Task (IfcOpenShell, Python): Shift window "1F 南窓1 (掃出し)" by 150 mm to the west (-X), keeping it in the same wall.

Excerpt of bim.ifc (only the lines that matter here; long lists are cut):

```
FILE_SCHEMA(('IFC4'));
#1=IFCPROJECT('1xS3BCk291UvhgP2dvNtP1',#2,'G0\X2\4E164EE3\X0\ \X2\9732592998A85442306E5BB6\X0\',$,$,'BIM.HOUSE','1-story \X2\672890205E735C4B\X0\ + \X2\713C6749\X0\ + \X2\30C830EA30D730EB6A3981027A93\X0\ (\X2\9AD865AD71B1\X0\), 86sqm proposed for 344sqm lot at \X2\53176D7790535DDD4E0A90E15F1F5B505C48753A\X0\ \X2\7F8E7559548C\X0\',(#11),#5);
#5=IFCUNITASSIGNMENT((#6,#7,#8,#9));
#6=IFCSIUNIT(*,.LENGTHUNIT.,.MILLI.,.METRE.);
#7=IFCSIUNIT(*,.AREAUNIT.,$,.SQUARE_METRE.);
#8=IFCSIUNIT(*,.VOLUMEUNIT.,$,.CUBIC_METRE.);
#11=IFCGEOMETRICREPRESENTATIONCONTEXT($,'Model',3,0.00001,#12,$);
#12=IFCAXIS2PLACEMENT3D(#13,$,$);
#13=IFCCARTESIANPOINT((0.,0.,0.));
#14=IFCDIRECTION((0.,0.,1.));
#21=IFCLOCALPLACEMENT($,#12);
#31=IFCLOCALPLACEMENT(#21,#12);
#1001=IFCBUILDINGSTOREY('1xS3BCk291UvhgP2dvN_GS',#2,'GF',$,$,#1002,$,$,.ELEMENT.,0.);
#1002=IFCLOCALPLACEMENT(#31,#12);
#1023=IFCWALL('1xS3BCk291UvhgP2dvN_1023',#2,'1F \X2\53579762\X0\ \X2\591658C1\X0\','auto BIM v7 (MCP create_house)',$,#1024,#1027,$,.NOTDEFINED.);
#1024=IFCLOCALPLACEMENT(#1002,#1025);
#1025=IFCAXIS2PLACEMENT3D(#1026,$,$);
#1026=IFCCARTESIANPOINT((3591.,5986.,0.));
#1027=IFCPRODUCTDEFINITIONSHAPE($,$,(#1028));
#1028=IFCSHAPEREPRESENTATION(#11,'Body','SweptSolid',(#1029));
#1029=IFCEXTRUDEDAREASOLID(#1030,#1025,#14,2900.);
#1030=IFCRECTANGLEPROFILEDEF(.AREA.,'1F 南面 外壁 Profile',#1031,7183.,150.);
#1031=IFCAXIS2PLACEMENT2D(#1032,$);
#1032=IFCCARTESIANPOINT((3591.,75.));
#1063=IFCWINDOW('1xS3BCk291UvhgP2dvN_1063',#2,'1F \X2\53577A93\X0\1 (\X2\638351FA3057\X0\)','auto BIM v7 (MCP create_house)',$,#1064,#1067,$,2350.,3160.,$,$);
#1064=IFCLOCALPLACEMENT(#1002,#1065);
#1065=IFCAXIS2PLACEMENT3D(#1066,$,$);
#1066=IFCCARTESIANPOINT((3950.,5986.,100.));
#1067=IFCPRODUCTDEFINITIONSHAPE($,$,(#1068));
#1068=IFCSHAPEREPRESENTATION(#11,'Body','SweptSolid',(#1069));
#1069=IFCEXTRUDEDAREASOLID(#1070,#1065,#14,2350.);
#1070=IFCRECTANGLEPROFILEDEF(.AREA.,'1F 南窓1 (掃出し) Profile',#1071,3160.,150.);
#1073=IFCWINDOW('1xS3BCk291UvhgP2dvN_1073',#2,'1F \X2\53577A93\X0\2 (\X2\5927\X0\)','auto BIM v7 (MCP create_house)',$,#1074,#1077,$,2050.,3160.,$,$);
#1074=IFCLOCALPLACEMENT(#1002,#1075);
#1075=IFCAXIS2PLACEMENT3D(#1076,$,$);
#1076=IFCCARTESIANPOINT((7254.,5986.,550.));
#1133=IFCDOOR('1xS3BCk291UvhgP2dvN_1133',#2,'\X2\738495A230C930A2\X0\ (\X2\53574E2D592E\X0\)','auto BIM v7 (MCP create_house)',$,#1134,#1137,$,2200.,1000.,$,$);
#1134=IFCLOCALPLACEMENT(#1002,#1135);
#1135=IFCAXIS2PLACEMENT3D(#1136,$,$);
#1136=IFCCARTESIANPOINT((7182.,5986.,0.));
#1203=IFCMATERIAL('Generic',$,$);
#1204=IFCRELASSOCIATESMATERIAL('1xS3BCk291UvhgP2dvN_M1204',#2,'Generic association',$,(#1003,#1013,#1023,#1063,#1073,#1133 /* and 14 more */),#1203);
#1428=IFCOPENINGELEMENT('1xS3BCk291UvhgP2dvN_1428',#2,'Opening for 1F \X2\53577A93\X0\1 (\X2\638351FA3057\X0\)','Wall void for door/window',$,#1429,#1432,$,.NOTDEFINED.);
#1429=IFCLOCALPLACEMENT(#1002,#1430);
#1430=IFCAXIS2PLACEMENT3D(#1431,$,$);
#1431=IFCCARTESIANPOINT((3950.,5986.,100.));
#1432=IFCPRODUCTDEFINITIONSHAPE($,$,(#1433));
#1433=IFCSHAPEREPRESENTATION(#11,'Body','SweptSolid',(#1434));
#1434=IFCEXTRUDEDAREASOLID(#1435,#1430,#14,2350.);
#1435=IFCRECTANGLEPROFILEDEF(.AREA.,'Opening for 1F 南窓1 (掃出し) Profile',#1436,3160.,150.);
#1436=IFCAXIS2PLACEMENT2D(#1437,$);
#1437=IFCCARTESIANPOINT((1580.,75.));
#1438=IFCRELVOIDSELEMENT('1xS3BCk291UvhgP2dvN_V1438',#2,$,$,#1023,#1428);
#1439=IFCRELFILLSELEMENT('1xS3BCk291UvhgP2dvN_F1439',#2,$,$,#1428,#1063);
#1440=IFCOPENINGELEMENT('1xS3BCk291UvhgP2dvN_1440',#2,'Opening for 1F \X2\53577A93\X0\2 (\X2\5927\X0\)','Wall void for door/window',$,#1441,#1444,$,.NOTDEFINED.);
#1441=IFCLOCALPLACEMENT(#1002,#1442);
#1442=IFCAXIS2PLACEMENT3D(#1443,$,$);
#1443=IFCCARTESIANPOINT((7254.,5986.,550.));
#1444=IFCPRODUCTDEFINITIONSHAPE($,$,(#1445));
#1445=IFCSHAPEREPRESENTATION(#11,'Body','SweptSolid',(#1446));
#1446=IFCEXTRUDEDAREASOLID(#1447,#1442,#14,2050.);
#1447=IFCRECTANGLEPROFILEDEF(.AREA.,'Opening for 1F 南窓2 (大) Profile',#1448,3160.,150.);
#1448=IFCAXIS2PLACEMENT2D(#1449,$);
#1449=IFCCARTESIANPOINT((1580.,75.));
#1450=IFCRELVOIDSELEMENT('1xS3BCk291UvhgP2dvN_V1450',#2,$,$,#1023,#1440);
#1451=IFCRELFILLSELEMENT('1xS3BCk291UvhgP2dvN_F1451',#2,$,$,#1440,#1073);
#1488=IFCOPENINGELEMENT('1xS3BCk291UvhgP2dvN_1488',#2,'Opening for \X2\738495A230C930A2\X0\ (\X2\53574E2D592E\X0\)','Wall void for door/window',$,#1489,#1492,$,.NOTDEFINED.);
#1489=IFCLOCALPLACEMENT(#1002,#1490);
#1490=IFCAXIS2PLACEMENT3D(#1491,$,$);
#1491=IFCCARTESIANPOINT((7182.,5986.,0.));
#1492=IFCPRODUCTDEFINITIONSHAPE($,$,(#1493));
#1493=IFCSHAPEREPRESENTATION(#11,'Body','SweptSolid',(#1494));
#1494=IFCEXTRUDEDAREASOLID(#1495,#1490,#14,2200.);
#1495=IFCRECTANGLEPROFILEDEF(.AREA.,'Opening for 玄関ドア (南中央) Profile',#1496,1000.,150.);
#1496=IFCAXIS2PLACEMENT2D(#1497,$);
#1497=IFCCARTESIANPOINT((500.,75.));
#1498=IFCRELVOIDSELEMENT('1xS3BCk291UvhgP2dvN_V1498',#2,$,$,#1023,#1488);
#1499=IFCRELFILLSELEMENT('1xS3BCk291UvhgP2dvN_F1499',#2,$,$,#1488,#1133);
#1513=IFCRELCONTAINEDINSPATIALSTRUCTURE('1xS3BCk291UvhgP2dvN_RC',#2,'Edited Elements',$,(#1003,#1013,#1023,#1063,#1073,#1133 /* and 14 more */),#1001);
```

```python
import ifcopenshell
import ifcopenshell.api.geometry
import ifcopenshell.util.placement

model = ifcopenshell.open("bim.ifc")

window = model.by_guid("1xS3BCk291UvhgP2dvN_1063")
opening = window.FillsVoids[0].RelatingOpeningElement
wall = opening.VoidsElements[0].RelatingBuildingElement

wall_matrix = ifcopenshell.util.placement.get_local_placement(wall.ObjectPlacement)
shift = wall_matrix[:3, 0] * -150.0
before = ifcopenshell.util.placement.get_local_placement(window.ObjectPlacement)[:3, 3].copy()

# The window is not placed relative to its opening, so move both.
for product in (opening, window):
    matrix = ifcopenshell.util.placement.get_local_placement(product.ObjectPlacement)
    matrix[:3, 3] += shift
    ifcopenshell.api.geometry.edit_object_placement(model, product=product, matrix=matrix, is_si=False)

after = ifcopenshell.util.placement.get_local_placement(window.ObjectPlacement)[:3, 3]
print("window moved by", (after - before).round(3) + 0.0)

model.write("bim_edited.ifc")
```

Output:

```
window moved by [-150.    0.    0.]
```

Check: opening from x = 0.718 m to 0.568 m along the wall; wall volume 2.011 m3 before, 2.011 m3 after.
